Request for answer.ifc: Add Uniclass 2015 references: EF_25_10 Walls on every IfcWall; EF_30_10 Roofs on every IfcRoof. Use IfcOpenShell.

First a look at what the model holds.

```python
import ifcopenshell

model = ifcopenshell.open("answer.ifc")
print(model.schema)
print("classifications:", [c.Name for c in model.by_type("IfcClassification")])
for ifc_class in ("IfcDoor", "IfcRoof", "IfcStair", "IfcWall", "IfcWindow"):
    print(ifc_class, len(model.by_type(ifc_class)))
```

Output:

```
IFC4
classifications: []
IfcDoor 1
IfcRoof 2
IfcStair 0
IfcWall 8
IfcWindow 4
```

```python
import ifcopenshell
import ifcopenshell.api.classification

model = ifcopenshell.open("answer.ifc")

system = ifcopenshell.api.classification.add_classification(model, classification="Uniclass 2015")

codes = {
    "IfcWall": ("EF_25_10", "Walls"),
    "IfcRoof": ("EF_30_10", "Roofs"),
}
for ifc_class, (code, name) in codes.items():
    products = model.by_type(ifc_class)
    ifcopenshell.api.classification.add_reference(
        model, products=products, classification=system, identification=code, name=name
    )
    print(code, len(products))

model.write("answer-out.ifc")
```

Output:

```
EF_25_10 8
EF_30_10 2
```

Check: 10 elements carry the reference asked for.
